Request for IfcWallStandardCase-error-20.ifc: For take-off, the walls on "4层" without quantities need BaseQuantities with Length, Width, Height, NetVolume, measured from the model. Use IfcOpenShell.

First a look at what the model holds.

```python
import ifcopenshell
import ifcopenshell.util.element
import ifcopenshell.util.unit

model = ifcopenshell.open("IfcWallStandardCase-error-20.ifc")
print(model.schema)
for unit_type in ("LENGTHUNIT", "AREAUNIT", "VOLUMEUNIT"):
    print(unit_type, ifcopenshell.util.unit.calculate_unit_scale(model, unit_type))
storey = next(s for s in model.by_type("IfcBuildingStorey") if s.Name == "4层")
walls = [e for e in ifcopenshell.util.element.get_decomposition(storey) if e.is_a("IfcWall")]
for e in sorted(walls, key=lambda e: e.id()):
    print(e.id(), e.is_a(), e.Name, list(ifcopenshell.util.element.get_psets(e, qtos_only=True)), sep=" | ")
```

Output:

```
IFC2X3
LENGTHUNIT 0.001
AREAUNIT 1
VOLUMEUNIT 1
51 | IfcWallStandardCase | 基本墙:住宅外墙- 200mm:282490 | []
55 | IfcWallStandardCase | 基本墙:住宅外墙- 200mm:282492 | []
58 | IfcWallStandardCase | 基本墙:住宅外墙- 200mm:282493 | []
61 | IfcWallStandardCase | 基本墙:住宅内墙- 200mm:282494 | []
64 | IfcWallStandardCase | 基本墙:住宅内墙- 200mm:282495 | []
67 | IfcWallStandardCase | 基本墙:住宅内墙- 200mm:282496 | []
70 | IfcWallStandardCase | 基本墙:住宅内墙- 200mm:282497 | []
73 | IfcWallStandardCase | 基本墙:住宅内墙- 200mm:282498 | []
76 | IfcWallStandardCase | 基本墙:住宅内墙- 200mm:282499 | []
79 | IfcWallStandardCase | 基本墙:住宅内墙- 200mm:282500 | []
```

```python
import ifcopenshell
import ifcopenshell.api.pset
import ifcopenshell.geom
import ifcopenshell.util.element
import ifcopenshell.util.shape
import ifcopenshell.util.unit

model = ifcopenshell.open("IfcWallStandardCase-error-20.ifc")
unit_scale = ifcopenshell.util.unit.calculate_unit_scale(model)
volume_scale = ifcopenshell.util.unit.calculate_unit_scale(model, "VOLUMEUNIT")
settings = ifcopenshell.geom.settings()

storey = next(s for s in model.by_type("IfcBuildingStorey") if s.Name == "4层")
walls = [e for e in ifcopenshell.util.element.get_decomposition(storey) if e.is_a("IfcWall")]

for e in sorted(walls, key=lambda e: e.id()):
    if ifcopenshell.util.element.get_psets(e, qtos_only=True, should_inherit=False):
        continue
    # Geometry comes back in metres, in the element's own axes.
    shape = ifcopenshell.geom.create_shape(settings, e)
    values = {
        "Length": ifcopenshell.util.shape.get_x(shape.geometry) / unit_scale,
        "Width": ifcopenshell.util.shape.get_y(shape.geometry) / unit_scale,
        "Height": ifcopenshell.util.shape.get_z(shape.geometry) / unit_scale,
        "NetVolume": ifcopenshell.util.shape.get_volume(shape.geometry) / volume_scale,
    }
    qto = ifcopenshell.api.pset.add_qto(model, product=e, name="BaseQuantities")
    ifcopenshell.api.pset.edit_qto(model, qto=qto, properties=values)
    print(e.id(), {k: round(v, 3) for k, v in values.items()})

model.write("IfcWallStandardCase-error-20_rev.ifc")
```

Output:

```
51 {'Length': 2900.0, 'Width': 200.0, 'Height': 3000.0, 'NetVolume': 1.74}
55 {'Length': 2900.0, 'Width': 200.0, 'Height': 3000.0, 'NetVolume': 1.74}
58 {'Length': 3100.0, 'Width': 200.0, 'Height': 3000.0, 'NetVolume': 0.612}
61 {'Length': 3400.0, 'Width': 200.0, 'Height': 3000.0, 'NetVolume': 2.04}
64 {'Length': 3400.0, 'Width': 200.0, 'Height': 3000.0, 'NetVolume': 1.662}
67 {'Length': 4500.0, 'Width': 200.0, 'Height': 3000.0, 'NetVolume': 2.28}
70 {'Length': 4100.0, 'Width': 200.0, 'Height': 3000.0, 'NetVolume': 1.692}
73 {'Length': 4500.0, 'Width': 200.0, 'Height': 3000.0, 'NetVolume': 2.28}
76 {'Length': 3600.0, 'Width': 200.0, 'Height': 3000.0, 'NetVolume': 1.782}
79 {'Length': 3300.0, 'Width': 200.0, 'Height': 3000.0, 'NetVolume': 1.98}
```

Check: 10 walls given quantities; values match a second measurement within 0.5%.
